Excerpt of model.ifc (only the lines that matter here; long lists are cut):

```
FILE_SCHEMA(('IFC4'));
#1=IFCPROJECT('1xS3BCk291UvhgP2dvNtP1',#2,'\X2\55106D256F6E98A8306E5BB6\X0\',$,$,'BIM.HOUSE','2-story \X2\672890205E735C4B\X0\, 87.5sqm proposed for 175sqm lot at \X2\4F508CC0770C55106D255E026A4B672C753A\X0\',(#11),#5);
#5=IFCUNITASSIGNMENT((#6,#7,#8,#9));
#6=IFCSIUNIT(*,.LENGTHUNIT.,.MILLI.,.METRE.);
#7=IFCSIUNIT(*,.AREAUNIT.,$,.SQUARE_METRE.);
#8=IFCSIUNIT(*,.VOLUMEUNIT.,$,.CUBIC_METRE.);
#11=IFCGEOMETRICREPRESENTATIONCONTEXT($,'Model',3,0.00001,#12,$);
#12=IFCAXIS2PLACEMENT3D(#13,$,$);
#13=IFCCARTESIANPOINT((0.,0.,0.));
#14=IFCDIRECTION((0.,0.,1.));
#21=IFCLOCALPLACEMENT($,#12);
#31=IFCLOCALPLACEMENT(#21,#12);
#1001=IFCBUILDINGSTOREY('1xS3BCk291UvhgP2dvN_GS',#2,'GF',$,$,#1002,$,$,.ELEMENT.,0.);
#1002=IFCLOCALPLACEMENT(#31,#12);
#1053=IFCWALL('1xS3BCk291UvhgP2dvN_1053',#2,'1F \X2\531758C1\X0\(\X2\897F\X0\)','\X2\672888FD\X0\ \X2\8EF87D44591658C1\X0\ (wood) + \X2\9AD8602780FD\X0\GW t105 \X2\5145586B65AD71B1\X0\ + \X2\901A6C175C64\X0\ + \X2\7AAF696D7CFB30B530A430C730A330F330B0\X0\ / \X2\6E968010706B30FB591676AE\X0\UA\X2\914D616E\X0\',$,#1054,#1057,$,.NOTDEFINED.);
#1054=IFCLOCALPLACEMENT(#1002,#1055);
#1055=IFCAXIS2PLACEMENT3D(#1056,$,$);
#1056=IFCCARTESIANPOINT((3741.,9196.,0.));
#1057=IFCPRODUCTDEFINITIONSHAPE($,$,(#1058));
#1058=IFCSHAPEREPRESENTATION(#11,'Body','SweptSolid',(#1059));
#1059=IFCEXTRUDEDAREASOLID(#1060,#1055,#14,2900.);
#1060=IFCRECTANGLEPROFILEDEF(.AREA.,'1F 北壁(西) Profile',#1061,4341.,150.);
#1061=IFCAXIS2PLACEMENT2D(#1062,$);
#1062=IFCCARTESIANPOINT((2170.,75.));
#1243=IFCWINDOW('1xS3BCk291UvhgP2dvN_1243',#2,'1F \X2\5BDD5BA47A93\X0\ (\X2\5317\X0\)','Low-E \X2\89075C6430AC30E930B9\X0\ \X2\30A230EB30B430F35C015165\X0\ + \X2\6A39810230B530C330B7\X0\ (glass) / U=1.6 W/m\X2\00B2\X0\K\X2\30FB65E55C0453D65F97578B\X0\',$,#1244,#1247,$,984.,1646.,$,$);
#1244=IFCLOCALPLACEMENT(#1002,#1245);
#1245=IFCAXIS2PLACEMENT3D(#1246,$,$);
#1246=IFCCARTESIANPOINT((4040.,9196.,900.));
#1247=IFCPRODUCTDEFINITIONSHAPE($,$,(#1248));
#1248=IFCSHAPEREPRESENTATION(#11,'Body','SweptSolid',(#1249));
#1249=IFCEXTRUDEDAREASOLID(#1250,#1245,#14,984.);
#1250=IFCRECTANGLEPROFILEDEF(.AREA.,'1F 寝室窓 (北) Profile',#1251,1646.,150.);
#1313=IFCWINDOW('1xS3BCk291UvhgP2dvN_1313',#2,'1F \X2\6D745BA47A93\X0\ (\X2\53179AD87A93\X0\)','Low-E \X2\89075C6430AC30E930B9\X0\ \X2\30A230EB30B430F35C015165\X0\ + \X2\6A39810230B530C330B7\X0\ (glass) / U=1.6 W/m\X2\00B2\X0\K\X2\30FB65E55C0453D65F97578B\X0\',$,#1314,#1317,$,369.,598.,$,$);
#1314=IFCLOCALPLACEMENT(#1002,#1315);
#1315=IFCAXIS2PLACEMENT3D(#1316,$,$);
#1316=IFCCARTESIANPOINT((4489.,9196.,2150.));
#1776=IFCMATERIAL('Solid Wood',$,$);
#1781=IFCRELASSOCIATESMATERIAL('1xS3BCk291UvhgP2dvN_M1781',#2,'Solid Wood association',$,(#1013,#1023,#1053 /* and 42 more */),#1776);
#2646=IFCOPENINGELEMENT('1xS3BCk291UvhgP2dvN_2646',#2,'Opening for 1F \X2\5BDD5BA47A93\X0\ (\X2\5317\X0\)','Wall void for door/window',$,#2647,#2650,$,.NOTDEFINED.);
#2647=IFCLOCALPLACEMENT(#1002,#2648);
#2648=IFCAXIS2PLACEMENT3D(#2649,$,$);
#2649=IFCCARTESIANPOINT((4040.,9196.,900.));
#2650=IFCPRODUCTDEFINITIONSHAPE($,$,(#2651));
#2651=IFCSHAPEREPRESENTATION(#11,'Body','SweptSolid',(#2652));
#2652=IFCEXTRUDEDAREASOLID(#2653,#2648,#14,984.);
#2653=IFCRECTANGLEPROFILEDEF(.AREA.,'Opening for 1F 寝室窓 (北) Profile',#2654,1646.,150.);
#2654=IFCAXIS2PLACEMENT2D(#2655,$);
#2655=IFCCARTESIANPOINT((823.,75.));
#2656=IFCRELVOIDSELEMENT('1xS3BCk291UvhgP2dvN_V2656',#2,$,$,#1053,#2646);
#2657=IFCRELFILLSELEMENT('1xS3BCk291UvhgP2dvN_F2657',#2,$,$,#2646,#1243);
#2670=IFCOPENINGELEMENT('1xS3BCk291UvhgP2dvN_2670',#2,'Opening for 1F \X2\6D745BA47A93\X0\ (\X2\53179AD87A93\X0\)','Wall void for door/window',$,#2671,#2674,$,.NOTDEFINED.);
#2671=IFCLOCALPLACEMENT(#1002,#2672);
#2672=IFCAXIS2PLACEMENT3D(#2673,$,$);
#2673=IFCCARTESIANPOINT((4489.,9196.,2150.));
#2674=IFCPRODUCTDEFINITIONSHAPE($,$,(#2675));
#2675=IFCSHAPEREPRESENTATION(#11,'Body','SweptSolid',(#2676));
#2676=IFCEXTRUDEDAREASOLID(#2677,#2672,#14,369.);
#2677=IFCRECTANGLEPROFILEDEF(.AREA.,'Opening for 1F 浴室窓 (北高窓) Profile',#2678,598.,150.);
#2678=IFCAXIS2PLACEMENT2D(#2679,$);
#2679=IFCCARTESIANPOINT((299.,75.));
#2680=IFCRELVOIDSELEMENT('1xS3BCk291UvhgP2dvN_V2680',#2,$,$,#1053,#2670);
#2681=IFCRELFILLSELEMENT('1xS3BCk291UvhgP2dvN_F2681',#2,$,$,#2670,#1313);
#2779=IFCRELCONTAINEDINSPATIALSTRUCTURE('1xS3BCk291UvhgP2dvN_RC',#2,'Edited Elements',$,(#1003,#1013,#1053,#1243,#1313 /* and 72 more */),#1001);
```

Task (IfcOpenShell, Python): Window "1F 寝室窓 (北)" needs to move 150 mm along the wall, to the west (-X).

```python
import ifcopenshell
import ifcopenshell.api.geometry
import ifcopenshell.util.placement
import ifcopenshell.util.unit

model = ifcopenshell.open("model.ifc")
unit_scale = ifcopenshell.util.unit.calculate_unit_scale(model)

window = model.by_guid("1xS3BCk291UvhgP2dvN_1243")
opening = window.FillsVoids[0].RelatingOpeningElement
wall = opening.VoidsElements[0].RelatingBuildingElement

wall_matrix = ifcopenshell.util.placement.get_local_placement(wall.ObjectPlacement)
shift = wall_matrix[:3, 0] * -0.15 / unit_scale
before = ifcopenshell.util.placement.get_local_placement(window.ObjectPlacement)[:3, 3].copy()

# The window is not placed relative to its opening, so move both.
for product in (opening, window):
    matrix = ifcopenshell.util.placement.get_local_placement(product.ObjectPlacement)
    matrix[:3, 3] += shift
    ifcopenshell.api.geometry.edit_object_placement(model, product=product, matrix=matrix, is_si=False)

after = ifcopenshell.util.placement.get_local_placement(window.ObjectPlacement)[:3, 3]
print("window moved by", (after - before).round(3) + 0.0)

model.write("model_v2.ifc")
```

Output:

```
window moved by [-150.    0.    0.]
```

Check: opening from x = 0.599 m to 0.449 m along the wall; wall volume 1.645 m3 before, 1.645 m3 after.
